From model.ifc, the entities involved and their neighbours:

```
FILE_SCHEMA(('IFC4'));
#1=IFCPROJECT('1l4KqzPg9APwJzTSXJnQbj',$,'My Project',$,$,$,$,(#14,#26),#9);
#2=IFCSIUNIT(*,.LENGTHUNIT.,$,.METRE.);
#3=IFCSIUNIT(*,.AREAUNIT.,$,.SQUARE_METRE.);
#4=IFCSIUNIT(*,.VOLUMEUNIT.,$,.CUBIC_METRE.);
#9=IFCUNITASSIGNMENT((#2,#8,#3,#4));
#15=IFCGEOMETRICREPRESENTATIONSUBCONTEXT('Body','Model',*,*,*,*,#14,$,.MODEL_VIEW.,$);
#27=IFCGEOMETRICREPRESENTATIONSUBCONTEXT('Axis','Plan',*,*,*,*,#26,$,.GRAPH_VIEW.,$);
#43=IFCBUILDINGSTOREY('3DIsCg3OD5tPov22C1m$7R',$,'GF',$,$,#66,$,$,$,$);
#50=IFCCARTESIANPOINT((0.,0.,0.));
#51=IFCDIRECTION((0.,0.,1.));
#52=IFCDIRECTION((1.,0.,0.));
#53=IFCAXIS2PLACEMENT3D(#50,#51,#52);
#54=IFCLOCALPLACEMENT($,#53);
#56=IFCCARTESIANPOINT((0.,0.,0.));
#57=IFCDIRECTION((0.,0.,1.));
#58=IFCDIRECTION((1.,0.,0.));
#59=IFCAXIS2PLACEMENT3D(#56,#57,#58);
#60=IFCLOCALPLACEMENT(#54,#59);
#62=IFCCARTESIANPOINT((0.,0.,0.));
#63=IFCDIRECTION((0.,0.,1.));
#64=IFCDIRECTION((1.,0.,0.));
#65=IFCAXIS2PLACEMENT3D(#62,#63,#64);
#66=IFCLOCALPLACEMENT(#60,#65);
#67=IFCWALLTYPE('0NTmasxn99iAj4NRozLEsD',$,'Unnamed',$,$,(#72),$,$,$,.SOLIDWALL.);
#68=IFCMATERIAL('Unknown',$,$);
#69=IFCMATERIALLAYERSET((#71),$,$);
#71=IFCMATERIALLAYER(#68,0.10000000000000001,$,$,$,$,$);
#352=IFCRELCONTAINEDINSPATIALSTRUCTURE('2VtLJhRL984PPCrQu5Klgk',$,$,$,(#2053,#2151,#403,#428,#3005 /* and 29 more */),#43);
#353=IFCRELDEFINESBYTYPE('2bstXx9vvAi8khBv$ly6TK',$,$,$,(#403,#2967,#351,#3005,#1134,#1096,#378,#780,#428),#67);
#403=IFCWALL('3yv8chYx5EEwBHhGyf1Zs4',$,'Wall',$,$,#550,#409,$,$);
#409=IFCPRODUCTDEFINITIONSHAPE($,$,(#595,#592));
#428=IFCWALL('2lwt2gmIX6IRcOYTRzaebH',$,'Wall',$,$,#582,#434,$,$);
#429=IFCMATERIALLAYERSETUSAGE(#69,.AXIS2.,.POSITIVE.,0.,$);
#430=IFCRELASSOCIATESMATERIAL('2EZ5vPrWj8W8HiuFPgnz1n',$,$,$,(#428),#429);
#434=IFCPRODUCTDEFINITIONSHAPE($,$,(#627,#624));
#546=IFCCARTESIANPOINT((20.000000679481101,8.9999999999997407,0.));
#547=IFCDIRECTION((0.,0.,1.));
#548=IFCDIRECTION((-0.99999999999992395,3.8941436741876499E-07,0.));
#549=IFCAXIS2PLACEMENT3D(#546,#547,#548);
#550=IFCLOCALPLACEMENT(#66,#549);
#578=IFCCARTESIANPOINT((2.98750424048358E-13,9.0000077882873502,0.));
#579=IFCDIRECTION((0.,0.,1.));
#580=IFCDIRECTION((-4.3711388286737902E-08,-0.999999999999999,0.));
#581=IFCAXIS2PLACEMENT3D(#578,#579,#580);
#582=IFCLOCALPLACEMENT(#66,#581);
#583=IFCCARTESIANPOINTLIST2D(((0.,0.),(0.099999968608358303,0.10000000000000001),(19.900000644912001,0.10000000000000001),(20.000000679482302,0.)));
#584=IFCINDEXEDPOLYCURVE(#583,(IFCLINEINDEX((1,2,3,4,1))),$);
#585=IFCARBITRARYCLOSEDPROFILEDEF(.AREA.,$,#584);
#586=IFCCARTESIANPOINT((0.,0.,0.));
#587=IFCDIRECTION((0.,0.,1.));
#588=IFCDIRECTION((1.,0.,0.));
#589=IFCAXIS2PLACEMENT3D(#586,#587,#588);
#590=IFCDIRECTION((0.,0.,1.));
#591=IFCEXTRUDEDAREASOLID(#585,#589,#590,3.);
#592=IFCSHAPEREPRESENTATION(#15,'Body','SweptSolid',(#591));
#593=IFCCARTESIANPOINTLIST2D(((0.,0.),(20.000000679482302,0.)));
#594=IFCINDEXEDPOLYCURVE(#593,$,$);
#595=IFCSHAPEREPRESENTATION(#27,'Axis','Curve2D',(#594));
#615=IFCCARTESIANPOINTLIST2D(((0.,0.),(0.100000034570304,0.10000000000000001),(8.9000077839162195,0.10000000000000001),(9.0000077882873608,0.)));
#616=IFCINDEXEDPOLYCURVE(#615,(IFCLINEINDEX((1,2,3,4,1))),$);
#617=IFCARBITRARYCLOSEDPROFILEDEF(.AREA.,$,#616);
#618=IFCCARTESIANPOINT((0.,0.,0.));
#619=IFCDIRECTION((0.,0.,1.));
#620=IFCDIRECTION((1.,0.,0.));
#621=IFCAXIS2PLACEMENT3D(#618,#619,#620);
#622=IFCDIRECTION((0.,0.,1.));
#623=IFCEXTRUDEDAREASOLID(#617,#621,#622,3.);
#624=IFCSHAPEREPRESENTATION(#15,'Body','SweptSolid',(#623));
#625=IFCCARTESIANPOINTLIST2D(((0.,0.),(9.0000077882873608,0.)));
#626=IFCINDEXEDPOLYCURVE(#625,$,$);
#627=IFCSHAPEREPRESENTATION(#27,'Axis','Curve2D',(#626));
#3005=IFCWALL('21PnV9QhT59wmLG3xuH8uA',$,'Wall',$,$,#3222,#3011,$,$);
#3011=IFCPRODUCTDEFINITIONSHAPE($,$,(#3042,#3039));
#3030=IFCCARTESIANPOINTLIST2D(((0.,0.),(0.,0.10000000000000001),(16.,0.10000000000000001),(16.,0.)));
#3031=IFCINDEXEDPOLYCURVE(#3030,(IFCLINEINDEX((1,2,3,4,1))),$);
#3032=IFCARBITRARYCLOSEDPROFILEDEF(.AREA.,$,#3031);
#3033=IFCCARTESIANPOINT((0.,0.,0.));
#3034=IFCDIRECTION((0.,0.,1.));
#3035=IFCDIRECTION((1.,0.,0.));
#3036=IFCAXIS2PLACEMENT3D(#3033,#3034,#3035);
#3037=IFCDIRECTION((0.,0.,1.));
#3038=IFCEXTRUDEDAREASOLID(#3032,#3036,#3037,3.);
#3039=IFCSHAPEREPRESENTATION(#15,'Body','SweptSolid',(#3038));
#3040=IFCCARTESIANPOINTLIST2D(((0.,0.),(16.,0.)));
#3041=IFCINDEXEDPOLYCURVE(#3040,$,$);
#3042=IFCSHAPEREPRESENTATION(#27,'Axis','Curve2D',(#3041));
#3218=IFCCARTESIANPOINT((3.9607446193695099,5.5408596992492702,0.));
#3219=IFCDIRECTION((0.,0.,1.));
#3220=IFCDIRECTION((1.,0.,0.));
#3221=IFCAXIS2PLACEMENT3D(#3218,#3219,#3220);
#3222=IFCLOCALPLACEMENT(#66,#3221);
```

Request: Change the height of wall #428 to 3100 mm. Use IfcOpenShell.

```python
import ifcopenshell
import ifcopenshell.geom
import ifcopenshell.util.representation
import ifcopenshell.util.shape
import ifcopenshell.util.unit

model = ifcopenshell.open("model.ifc")
unit_scale = ifcopenshell.util.unit.calculate_unit_scale(model)
settings = ifcopenshell.geom.settings()


def volume(element):
    """Net volume in cubic metres, openings subtracted."""
    shape = ifcopenshell.geom.create_shape(settings, element)
    return ifcopenshell.util.shape.get_volume(shape.geometry)


wall = model.by_guid("2lwt2gmIX6IRcOYTRzaebH")
before = volume(wall)

body = ifcopenshell.util.representation.get_representation(wall, "Model", "Body")
solid = body.Items[0]
old_height = solid.Depth
solid.Depth = 3.1 / unit_scale
after = volume(wall)

print(f"height {old_height:g} -> {solid.Depth:g}, volume {before:.3f} -> {after:.3f} m3")

model.write("model_v2.ifc")
```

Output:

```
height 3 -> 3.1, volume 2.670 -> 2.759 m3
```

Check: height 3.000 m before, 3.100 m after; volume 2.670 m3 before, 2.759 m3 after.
